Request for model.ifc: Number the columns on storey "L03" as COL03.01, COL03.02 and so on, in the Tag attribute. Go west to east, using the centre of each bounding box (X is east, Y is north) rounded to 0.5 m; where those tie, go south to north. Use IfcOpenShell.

First a look at what the model holds.

```python
import ifcopenshell
import ifcopenshell.util.element
import ifcopenshell.util.placement

model = ifcopenshell.open("model.ifc")
print(model.schema)
storey = next(s for s in model.by_type("IfcBuildingStorey") if s.Name == "L03")
columns = [e for e in ifcopenshell.util.element.get_decomposition(storey) if e.is_a("IfcColumn")]
for e in sorted(columns, key=lambda e: e.id()):
    origin = ifcopenshell.util.placement.get_local_placement(e.ObjectPlacement)[:3, 3]
    print(e.id(), e.Tag, e.Name, origin.round(2) + 0.0, sep=" | ")
```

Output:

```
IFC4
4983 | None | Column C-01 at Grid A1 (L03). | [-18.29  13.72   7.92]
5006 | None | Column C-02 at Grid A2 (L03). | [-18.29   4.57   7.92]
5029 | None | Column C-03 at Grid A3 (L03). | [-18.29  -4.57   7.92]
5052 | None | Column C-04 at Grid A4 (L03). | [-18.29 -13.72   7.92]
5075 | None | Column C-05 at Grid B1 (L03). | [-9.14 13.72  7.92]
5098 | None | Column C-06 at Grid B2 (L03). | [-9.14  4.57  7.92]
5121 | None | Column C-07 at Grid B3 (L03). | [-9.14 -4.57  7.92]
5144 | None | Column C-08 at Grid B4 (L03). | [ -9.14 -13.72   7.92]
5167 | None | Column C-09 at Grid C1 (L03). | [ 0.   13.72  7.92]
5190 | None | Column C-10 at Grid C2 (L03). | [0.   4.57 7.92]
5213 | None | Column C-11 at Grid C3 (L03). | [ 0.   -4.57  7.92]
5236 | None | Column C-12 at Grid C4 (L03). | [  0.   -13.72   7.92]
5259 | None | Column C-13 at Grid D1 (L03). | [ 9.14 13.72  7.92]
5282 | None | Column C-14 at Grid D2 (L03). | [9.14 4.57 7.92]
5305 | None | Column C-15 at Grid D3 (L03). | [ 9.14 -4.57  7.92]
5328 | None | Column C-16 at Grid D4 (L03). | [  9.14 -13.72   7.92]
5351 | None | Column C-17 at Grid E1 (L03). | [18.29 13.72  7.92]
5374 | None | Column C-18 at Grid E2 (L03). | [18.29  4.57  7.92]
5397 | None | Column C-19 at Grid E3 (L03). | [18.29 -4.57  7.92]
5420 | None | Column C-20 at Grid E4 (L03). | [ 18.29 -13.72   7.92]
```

```python
import ifcopenshell
import ifcopenshell.geom
import ifcopenshell.util.element
import ifcopenshell.util.shape

model = ifcopenshell.open("model.ifc")
settings = ifcopenshell.geom.settings()
settings.set("use-world-coords", True)


def centre(element):
    shape = ifcopenshell.geom.create_shape(settings, element)
    return ifcopenshell.util.shape.get_bbox_centroid(shape.geometry)


storey = next(s for s in model.by_type("IfcBuildingStorey") if s.Name == "L03")
columns = [e for e in ifcopenshell.util.element.get_decomposition(storey) if e.is_a("IfcColumn")]

# Insertion points can sit at a corner or the storey origin, so sort by the geometry (in metres).
centres = {e: centre(e) for e in columns}
columns.sort(key=lambda e: (round(centres[e][0] / 0.5), centres[e][1]))

for i, e in enumerate(columns, start=1):
    number = f"COL03.{i:02d}"
    e.Tag = number
    print(e.id(), number)

model.write("model_v2.ifc")
```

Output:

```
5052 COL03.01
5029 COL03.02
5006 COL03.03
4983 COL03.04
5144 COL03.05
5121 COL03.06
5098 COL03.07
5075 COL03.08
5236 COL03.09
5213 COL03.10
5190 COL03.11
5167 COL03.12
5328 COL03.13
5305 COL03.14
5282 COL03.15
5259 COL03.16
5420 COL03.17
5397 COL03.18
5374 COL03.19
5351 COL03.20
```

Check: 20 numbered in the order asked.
